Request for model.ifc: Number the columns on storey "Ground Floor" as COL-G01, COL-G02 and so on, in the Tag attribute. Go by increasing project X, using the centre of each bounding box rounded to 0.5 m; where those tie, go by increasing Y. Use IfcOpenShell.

First a look at what the model holds.

```python
import ifcopenshell
import ifcopenshell.util.element
import ifcopenshell.util.placement

model = ifcopenshell.open("model.ifc")
print(model.schema)
storey = next(s for s in model.by_type("IfcBuildingStorey") if s.Name == "Ground Floor")
columns = [e for e in ifcopenshell.util.element.get_decomposition(storey) if e.is_a("IfcColumn")]
for e in sorted(columns, key=lambda e: e.id()):
    origin = ifcopenshell.util.placement.get_local_placement(e.ObjectPlacement)[:3, 3]
    print(e.id(), e.Tag, e.Name, origin.round(2) + 0.0, sep=" | ")
```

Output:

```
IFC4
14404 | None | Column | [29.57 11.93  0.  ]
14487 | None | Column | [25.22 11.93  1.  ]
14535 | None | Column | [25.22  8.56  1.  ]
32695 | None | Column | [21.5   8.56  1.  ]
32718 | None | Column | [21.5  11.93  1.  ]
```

```python
import ifcopenshell
import ifcopenshell.geom
import ifcopenshell.util.element
import ifcopenshell.util.shape

model = ifcopenshell.open("model.ifc")
settings = ifcopenshell.geom.settings()
settings.set("use-world-coords", True)


def centre(element):
    shape = ifcopenshell.geom.create_shape(settings, element)
    return ifcopenshell.util.shape.get_bbox_centroid(shape.geometry)


storey = next(s for s in model.by_type("IfcBuildingStorey") if s.Name == "Ground Floor")
columns = [e for e in ifcopenshell.util.element.get_decomposition(storey) if e.is_a("IfcColumn")]

# Insertion points can sit at a corner or the storey origin, so sort by the geometry (in metres).
centres = {e: centre(e) for e in columns}
columns.sort(key=lambda e: (round(centres[e][0] / 0.5), centres[e][1]))

for i, e in enumerate(columns, start=1):
    number = f"COL-G{i:02d}"
    e.Tag = number
    print(e.id(), number)

model.write("model_v2.ifc")
```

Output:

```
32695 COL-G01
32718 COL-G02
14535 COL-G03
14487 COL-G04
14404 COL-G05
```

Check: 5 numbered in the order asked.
